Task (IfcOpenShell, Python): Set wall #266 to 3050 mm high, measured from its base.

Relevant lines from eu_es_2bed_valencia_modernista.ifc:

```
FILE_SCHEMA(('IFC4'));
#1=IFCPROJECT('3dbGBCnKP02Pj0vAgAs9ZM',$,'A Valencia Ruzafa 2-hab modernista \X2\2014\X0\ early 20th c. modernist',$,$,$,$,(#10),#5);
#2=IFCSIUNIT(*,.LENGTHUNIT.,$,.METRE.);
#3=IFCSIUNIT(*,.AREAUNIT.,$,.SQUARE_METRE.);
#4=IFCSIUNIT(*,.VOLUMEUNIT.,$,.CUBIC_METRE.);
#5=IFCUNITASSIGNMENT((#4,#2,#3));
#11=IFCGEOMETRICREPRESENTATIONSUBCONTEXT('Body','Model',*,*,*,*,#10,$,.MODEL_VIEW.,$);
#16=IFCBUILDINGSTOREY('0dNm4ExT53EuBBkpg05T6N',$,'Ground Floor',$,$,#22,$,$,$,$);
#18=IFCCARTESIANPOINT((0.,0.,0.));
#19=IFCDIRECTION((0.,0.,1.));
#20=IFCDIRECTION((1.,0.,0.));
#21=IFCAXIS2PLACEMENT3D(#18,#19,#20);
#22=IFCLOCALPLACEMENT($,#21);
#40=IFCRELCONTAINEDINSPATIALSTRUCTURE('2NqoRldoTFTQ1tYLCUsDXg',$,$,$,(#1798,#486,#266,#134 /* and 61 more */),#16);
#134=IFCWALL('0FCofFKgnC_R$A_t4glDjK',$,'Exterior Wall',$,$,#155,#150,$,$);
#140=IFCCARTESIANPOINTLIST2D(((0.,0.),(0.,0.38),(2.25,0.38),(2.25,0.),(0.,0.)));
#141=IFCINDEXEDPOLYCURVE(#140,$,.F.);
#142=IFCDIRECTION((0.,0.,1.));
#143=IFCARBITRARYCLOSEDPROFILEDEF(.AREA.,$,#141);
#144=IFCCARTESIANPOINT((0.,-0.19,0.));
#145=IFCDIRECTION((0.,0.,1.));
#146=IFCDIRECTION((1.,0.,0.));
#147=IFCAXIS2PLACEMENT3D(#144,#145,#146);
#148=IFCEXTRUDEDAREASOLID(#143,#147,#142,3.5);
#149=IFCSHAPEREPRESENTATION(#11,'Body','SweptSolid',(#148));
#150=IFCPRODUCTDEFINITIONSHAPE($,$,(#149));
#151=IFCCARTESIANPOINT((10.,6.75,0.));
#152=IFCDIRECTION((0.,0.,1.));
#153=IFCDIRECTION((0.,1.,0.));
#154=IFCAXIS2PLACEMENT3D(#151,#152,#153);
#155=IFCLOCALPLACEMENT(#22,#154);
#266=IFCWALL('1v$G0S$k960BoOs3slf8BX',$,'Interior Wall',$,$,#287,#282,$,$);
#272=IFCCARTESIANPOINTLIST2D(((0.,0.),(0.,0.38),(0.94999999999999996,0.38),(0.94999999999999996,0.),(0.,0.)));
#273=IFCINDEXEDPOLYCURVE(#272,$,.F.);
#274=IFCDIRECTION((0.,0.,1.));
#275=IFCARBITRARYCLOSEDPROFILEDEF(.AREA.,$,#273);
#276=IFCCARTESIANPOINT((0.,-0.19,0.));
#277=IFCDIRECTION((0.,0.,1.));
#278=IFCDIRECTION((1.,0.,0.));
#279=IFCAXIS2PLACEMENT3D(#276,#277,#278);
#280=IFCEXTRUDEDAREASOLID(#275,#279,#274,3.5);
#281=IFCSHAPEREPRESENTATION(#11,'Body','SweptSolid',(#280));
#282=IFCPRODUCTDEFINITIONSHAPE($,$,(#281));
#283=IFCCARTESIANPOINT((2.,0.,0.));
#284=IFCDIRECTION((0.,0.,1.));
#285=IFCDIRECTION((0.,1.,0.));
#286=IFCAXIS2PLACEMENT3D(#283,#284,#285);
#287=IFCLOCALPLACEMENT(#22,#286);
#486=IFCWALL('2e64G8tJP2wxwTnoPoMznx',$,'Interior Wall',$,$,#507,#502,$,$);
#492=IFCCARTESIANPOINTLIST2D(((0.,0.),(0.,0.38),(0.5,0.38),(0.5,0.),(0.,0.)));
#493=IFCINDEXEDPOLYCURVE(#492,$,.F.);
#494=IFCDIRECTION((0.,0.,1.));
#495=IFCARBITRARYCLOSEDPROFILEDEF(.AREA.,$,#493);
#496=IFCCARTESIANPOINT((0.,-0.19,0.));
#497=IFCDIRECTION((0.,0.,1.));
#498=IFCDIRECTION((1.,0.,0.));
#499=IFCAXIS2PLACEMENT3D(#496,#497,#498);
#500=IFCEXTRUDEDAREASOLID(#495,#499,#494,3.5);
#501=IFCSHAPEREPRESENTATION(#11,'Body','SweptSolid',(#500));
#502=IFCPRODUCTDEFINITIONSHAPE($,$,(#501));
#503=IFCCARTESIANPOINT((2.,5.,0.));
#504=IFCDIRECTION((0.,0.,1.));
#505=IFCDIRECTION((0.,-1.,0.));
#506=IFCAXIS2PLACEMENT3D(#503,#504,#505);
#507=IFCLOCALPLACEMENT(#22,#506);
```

```python
import ifcopenshell
import ifcopenshell.geom
import ifcopenshell.util.representation
import ifcopenshell.util.shape
import ifcopenshell.util.unit

model = ifcopenshell.open("eu_es_2bed_valencia_modernista.ifc")
unit_scale = ifcopenshell.util.unit.calculate_unit_scale(model)
settings = ifcopenshell.geom.settings()


def volume(element):
    """Net volume in cubic metres, openings subtracted."""
    shape = ifcopenshell.geom.create_shape(settings, element)
    return ifcopenshell.util.shape.get_volume(shape.geometry)


wall = model.by_guid("1v$G0S$k960BoOs3slf8BX")
before = volume(wall)

body = ifcopenshell.util.representation.get_representation(wall, "Model", "Body")
solid = body.Items[0]
old_height = solid.Depth
solid.Depth = 3.05 / unit_scale
after = volume(wall)

print(f"height {old_height:g} -> {solid.Depth:g}, volume {before:.3f} -> {after:.3f} m3")

model.write("eu_es_2bed_valencia_modernista_edited.ifc")
```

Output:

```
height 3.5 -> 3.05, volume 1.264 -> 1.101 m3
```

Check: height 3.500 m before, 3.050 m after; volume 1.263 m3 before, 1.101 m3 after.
